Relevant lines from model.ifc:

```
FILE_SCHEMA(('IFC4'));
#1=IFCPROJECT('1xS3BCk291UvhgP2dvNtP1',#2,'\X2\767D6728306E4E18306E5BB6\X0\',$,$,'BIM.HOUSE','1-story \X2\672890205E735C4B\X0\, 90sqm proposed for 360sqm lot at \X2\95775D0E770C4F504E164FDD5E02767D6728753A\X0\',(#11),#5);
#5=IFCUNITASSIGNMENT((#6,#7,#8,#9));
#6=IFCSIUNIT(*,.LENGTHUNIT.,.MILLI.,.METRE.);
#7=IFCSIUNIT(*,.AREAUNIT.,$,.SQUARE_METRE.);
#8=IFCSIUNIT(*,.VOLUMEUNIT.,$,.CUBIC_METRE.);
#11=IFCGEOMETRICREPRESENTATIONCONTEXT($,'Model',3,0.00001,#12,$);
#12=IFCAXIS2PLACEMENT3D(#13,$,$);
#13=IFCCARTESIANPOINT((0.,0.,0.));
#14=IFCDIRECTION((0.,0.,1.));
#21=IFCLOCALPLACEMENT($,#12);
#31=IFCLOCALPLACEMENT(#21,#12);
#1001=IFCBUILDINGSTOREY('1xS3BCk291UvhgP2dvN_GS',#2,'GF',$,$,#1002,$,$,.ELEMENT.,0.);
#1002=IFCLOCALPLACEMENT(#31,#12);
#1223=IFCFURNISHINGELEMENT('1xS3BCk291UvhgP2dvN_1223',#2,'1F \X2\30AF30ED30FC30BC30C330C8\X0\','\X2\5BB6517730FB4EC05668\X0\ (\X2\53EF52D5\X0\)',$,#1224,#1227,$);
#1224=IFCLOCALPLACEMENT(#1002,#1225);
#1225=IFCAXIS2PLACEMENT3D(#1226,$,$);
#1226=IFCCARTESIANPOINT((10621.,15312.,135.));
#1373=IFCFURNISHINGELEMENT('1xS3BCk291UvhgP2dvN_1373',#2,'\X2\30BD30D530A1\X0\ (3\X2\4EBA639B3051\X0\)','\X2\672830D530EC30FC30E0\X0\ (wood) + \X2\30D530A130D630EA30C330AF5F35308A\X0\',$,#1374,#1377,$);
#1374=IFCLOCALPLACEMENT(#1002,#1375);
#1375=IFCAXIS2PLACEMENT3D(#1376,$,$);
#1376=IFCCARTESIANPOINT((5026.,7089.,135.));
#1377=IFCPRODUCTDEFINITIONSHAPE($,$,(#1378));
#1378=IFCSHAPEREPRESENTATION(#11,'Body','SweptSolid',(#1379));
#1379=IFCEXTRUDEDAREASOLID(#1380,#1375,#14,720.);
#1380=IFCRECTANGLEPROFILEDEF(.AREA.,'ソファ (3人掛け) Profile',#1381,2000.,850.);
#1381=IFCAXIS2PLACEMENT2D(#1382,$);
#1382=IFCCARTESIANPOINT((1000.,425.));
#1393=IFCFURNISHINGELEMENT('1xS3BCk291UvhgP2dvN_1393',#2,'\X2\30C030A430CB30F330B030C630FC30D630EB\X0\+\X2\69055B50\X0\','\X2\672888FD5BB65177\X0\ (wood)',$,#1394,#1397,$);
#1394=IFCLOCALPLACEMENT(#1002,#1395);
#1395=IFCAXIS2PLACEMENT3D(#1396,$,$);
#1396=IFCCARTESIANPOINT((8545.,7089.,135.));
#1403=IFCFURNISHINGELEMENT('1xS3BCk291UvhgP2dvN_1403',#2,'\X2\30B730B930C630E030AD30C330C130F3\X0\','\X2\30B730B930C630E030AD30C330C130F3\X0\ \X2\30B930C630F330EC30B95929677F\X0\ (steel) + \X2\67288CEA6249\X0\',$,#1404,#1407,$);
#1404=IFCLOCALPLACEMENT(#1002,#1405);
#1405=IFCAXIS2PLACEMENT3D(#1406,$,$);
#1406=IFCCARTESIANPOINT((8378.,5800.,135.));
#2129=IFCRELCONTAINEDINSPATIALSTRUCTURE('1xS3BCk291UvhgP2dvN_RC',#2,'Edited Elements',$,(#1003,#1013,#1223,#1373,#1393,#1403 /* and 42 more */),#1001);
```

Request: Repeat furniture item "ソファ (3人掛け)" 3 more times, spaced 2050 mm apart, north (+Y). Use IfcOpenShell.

```python
import numpy as np
import ifcopenshell
import ifcopenshell.api.geometry
import ifcopenshell.api.root
import ifcopenshell.util.element
import ifcopenshell.util.placement
import ifcopenshell.util.unit

model = ifcopenshell.open("model.ifc")
unit_scale = ifcopenshell.util.unit.calculate_unit_scale(model)


def reuse_history(source, copy):
    """copy_class also copies each property set's owner history, people and application; keep the originals."""
    for rel in copy.IsDefinedBy:
        if rel.is_a("IfcRelDefinesByProperties") and (history := rel.RelatingPropertyDefinition.OwnerHistory):
            rel.RelatingPropertyDefinition.OwnerHistory = source.OwnerHistory
            ifcopenshell.util.element.remove_deep2(model, history)


source = model.by_id(1373)
base = ifcopenshell.util.placement.get_local_placement(source.ObjectPlacement)
step = np.array([0.0, 1.0, 0.0]) * 2.05 / unit_scale

for i in range(1, 4):
    copy = ifcopenshell.api.root.copy_class(model, product=source)
    copy.Representation = ifcopenshell.util.element.copy_deep(
        model, source.Representation, exclude=["IfcGeometricRepresentationContext", "IfcRepresentationMap"]
    )
    reuse_history(source, copy)
    matrix = base.copy()
    matrix[:3, 3] += i * step
    print("added at", matrix[:3, 3].round(3) + 0.0)
    ifcopenshell.api.geometry.edit_object_placement(model, product=copy, matrix=matrix, is_si=False)

model.write("model_rev.ifc")
```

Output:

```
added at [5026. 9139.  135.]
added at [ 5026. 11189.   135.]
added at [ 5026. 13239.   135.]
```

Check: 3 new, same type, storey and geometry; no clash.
